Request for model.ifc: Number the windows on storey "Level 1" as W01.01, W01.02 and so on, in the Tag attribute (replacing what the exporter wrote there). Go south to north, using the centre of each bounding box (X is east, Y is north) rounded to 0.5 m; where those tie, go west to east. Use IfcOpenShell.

First a look at what the model holds.

```python
import ifcopenshell
import ifcopenshell.util.element
import ifcopenshell.util.placement

model = ifcopenshell.open("model.ifc")
print(model.schema)
storey = next(s for s in model.by_type("IfcBuildingStorey") if s.Name == "Level 1")
windows = [e for e in ifcopenshell.util.element.get_decomposition(storey) if e.is_a("IfcWindow")]
for e in sorted(windows, key=lambda e: e.id()):
    origin = ifcopenshell.util.placement.get_local_placement(e.ObjectPlacement)[:3, 3]
    print(e.id(), e.Tag, e.Name, origin.round(2) + 0.0, sep=" | ")
```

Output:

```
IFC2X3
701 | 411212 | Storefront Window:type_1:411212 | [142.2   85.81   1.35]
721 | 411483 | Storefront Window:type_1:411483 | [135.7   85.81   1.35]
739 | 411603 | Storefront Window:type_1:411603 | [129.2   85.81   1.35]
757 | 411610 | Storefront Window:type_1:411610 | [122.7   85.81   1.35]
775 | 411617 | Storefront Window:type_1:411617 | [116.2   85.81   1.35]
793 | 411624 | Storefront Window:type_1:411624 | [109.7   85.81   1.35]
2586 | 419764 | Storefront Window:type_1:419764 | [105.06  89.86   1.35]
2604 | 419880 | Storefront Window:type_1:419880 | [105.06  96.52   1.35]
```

```python
import ifcopenshell
import ifcopenshell.geom
import ifcopenshell.util.element
import ifcopenshell.util.shape

model = ifcopenshell.open("model.ifc")
settings = ifcopenshell.geom.settings()
settings.set("use-world-coords", True)


def centre(element):
    shape = ifcopenshell.geom.create_shape(settings, element)
    return ifcopenshell.util.shape.get_bbox_centroid(shape.geometry)


storey = next(s for s in model.by_type("IfcBuildingStorey") if s.Name == "Level 1")
windows = [e for e in ifcopenshell.util.element.get_decomposition(storey) if e.is_a("IfcWindow")]

# Insertion points can sit at a corner or the storey origin, so sort by the geometry (in metres).
centres = {e: centre(e) for e in windows}
windows.sort(key=lambda e: (round(centres[e][1] / 0.5), centres[e][0]))

for i, e in enumerate(windows, start=1):
    number = f"W01.{i:02d}"
    e.Tag = number
    print(e.id(), number)

model.write("model_edited.ifc")
```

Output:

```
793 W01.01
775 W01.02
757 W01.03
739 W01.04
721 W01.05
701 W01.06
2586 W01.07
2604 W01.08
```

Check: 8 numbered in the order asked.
